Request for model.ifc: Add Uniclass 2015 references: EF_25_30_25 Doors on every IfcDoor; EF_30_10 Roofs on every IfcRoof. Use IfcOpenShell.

First a look at what the model holds.

```python
import ifcopenshell

model = ifcopenshell.open("model.ifc")
print(model.schema)
print("classifications:", [c.Name for c in model.by_type("IfcClassification")])
for ifc_class in ("IfcDoor", "IfcRoof", "IfcStair", "IfcWall", "IfcWindow"):
    print(ifc_class, len(model.by_type(ifc_class)))
```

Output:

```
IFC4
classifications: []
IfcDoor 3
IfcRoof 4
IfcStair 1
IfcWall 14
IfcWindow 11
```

```python
import ifcopenshell
import ifcopenshell.api.classification

model = ifcopenshell.open("model.ifc")

system = ifcopenshell.api.classification.add_classification(model, classification="Uniclass 2015")

codes = {
    "IfcDoor": ("EF_25_30_25", "Doors"),
    "IfcRoof": ("EF_30_10", "Roofs"),
}
for ifc_class, (code, name) in codes.items():
    products = model.by_type(ifc_class)
    ifcopenshell.api.classification.add_reference(
        model, products=products, classification=system, identification=code, name=name
    )
    print(code, len(products))

model.write("model_edited.ifc")
```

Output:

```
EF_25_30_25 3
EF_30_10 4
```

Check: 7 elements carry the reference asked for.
